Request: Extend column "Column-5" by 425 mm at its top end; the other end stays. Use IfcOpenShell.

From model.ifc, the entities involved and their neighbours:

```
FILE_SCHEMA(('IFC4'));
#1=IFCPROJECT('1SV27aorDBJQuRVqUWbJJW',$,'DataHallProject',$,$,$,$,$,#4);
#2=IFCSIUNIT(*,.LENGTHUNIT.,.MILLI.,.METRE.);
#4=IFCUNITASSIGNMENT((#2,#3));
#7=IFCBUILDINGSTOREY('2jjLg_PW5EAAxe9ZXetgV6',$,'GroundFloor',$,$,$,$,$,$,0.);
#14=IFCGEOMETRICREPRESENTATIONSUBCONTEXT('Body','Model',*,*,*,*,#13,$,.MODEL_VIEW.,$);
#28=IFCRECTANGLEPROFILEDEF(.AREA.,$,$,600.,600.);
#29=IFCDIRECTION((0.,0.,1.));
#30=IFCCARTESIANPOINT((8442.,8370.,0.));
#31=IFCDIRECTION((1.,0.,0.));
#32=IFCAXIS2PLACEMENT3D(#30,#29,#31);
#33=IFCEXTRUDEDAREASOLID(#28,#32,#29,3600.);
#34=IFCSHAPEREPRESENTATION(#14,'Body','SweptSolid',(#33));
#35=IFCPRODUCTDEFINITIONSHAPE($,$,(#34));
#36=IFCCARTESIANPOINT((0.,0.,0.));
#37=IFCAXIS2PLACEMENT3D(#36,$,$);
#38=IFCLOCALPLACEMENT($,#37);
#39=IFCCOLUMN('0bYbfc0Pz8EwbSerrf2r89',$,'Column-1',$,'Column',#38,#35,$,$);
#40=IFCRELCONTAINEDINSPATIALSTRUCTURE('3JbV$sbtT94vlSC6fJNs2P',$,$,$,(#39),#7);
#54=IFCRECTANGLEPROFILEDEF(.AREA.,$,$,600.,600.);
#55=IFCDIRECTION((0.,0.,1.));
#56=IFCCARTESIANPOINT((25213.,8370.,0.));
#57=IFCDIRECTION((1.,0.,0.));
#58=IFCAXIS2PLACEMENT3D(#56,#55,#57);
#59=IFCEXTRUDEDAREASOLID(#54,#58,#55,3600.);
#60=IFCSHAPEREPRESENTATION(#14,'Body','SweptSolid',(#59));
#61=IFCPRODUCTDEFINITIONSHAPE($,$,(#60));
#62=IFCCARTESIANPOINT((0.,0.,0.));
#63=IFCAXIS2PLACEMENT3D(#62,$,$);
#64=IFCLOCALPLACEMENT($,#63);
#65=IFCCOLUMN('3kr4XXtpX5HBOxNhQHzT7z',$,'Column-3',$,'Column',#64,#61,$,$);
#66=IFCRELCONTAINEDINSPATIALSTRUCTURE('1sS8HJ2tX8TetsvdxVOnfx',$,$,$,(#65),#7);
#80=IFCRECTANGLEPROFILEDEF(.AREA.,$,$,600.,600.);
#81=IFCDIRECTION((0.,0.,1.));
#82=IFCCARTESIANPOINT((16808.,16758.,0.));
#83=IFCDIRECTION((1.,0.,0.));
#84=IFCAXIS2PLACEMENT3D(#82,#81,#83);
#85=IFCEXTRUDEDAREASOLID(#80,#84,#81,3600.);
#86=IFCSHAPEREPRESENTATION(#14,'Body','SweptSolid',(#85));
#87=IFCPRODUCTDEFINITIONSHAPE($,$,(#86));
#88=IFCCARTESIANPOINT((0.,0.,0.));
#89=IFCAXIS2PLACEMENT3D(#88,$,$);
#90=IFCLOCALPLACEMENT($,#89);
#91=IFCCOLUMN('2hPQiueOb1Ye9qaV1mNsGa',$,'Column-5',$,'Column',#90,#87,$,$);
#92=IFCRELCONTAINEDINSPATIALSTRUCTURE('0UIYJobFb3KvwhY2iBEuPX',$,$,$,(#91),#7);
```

```python
import ifcopenshell
import ifcopenshell.util.representation
import ifcopenshell.util.unit

model = ifcopenshell.open("model.ifc")
unit_scale = ifcopenshell.util.unit.calculate_unit_scale(model)

member = model.by_id(91)
change = 0.425 / unit_scale

# The extrusion runs towards the end named, so only its depth changes.
body = ifcopenshell.util.representation.get_representation(member, "Model", "Body")
solid = body.Items[0]
old_length = solid.Depth
solid.Depth += change

print(f"length {old_length:g} -> {solid.Depth:g}")

model.write("model_v2.ifc")
```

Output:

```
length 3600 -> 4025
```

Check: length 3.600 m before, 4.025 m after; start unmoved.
